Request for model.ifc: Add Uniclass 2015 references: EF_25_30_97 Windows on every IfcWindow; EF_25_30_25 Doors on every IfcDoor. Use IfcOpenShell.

First a look at what the model holds.

```python
import ifcopenshell

model = ifcopenshell.open("model.ifc")
print(model.schema)
print("classifications:", [c.Name for c in model.by_type("IfcClassification")])
for ifc_class in ("IfcDoor", "IfcRoof", "IfcStair", "IfcWall", "IfcWindow"):
    print(ifc_class, len(model.by_type(ifc_class)))
```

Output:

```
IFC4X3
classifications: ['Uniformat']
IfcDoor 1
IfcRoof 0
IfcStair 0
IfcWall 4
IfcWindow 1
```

```python
import ifcopenshell
import ifcopenshell.api.classification

model = ifcopenshell.open("model.ifc")

system = ifcopenshell.api.classification.add_classification(model, classification="Uniclass 2015")

codes = {
    "IfcWindow": ("EF_25_30_97", "Windows"),
    "IfcDoor": ("EF_25_30_25", "Doors"),
}
for ifc_class, (code, name) in codes.items():
    products = model.by_type(ifc_class)
    ifcopenshell.api.classification.add_reference(
        model, products=products, classification=system, identification=code, name=name
    )
    print(code, len(products))

model.write("model_updated.ifc")
```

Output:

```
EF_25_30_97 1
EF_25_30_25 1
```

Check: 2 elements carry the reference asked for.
